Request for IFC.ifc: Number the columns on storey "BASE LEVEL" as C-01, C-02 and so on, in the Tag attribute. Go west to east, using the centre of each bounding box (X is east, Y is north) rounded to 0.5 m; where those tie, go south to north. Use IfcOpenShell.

First a look at what the model holds.

```python
import ifcopenshell
import ifcopenshell.util.element
import ifcopenshell.util.placement

model = ifcopenshell.open("IFC.ifc")
print(model.schema)
storey = next(s for s in model.by_type("IfcBuildingStorey") if s.Name == "BASE LEVEL")
columns = [e for e in ifcopenshell.util.element.get_decomposition(storey) if e.is_a("IfcColumn")]
for e in sorted(columns, key=lambda e: e.id()):
    origin = ifcopenshell.util.placement.get_local_placement(e.ObjectPlacement)[:3, 3]
    print(e.id(), e.Tag, e.Name, origin.round(2) + 0.0, sep=" | ")
```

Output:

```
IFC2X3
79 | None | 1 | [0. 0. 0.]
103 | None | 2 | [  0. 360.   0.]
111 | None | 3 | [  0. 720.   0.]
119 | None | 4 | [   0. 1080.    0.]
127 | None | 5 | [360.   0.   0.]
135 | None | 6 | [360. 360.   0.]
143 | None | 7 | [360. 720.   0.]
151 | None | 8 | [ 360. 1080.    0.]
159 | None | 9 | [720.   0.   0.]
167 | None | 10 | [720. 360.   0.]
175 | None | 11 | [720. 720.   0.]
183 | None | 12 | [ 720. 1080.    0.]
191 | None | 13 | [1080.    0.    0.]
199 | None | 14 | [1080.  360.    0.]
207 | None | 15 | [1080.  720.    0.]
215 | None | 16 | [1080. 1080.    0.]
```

```python
import ifcopenshell
import ifcopenshell.geom
import ifcopenshell.util.element
import ifcopenshell.util.shape

model = ifcopenshell.open("IFC.ifc")
settings = ifcopenshell.geom.settings()
settings.set("use-world-coords", True)


def centre(element):
    shape = ifcopenshell.geom.create_shape(settings, element)
    return ifcopenshell.util.shape.get_bbox_centroid(shape.geometry)


storey = next(s for s in model.by_type("IfcBuildingStorey") if s.Name == "BASE LEVEL")
columns = [e for e in ifcopenshell.util.element.get_decomposition(storey) if e.is_a("IfcColumn")]

# Insertion points can sit at a corner or the storey origin, so sort by the geometry (in metres).
centres = {e: centre(e) for e in columns}
columns.sort(key=lambda e: (round(centres[e][0] / 0.5), centres[e][1]))

for i, e in enumerate(columns, start=1):
    number = f"C-{i:02d}"
    e.Tag = number
    print(e.id(), number)

model.write("IFC-out.ifc")
```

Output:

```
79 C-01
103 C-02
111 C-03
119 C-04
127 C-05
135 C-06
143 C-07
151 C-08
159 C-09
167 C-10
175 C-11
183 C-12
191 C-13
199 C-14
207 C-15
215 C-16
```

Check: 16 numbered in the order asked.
